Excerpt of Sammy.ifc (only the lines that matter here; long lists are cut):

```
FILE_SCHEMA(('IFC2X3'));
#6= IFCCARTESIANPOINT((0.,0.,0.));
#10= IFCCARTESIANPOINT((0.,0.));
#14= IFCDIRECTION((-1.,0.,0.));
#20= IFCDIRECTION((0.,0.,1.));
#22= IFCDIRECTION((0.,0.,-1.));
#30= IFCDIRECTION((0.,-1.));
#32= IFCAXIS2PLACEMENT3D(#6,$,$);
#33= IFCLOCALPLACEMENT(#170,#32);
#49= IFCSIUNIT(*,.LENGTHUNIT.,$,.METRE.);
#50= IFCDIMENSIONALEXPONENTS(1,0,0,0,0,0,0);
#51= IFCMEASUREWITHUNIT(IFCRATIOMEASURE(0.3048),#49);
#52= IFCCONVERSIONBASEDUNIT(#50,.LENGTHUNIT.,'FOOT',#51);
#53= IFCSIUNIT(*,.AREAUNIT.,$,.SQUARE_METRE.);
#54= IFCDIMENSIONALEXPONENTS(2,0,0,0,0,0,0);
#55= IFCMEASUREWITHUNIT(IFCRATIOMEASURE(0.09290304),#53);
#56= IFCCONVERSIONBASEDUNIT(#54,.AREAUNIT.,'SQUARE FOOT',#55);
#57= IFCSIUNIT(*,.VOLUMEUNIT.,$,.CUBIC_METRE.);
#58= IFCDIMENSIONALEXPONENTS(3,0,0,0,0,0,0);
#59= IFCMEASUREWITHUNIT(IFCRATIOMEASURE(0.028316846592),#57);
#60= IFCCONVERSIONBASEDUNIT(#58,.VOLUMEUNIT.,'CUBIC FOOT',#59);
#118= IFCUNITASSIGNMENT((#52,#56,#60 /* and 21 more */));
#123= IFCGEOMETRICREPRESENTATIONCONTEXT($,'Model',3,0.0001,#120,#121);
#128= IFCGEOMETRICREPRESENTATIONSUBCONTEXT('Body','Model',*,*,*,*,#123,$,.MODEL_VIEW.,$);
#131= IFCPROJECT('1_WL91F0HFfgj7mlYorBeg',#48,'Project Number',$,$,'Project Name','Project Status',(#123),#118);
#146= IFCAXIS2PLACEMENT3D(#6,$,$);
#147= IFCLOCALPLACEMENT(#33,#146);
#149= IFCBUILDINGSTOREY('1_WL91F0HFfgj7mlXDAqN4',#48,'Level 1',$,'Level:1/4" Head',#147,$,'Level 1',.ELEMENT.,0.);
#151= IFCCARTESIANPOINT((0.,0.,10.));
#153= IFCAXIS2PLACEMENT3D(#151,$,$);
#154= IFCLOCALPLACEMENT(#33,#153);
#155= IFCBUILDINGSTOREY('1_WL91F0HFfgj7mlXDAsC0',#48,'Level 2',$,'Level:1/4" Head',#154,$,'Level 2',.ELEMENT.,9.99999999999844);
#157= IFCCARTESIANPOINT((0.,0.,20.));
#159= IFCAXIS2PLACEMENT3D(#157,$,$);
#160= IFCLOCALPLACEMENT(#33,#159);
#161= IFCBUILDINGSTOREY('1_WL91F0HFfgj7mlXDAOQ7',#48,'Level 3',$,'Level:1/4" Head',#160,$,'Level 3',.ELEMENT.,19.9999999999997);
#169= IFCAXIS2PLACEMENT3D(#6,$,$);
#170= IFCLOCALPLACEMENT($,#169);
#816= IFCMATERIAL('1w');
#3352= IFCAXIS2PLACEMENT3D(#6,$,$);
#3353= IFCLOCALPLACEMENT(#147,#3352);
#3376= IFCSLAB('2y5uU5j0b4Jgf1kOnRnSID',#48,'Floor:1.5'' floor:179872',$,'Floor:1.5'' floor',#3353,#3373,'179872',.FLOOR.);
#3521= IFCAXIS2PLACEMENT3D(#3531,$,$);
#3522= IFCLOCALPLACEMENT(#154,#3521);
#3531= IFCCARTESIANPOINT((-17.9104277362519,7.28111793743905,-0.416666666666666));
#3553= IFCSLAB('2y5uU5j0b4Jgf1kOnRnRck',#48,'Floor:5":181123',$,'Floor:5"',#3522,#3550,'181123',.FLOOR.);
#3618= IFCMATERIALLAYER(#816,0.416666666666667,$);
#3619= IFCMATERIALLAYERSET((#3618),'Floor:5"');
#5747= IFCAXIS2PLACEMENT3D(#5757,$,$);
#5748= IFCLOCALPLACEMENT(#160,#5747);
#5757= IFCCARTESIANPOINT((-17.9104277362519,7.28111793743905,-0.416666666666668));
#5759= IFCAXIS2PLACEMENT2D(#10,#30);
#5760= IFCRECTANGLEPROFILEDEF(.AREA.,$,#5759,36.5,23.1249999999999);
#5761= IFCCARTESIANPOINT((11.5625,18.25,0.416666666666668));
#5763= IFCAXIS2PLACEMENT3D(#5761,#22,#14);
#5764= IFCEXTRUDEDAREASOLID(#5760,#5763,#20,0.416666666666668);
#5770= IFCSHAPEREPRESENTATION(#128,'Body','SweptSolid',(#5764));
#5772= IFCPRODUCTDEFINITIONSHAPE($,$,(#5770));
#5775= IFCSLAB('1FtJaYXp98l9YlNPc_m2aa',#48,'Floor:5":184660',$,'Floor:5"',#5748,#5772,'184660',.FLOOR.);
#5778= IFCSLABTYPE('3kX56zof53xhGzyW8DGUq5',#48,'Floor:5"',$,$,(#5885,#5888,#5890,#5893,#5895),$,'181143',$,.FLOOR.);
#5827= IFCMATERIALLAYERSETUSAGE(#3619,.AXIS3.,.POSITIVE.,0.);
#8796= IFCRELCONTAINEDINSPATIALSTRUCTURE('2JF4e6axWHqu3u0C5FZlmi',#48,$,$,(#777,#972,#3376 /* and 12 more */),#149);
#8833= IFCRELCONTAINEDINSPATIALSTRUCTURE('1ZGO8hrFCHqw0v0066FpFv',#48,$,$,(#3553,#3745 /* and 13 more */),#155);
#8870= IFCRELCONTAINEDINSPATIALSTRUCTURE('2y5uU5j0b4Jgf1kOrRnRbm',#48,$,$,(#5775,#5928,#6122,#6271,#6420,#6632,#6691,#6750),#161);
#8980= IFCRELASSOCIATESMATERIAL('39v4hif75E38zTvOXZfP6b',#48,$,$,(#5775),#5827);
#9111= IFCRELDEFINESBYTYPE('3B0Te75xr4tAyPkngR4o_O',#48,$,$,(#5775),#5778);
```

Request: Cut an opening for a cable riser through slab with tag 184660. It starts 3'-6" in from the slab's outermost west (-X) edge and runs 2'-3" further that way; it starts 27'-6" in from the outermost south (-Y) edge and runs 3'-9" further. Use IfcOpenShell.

```python
import numpy as np
import ifcopenshell
import ifcopenshell.api.feature
import ifcopenshell.api.geometry
import ifcopenshell.api.root
import ifcopenshell.geom
import ifcopenshell.util.placement
import ifcopenshell.util.representation
import ifcopenshell.util.shape
import ifcopenshell.util.unit

model = ifcopenshell.open("Sammy.ifc")
unit_scale = ifcopenshell.util.unit.calculate_unit_scale(model)
settings = ifcopenshell.geom.settings()


def volume(element):
    """Net volume in cubic metres, openings subtracted."""
    shape = ifcopenshell.geom.create_shape(settings, element)
    return ifcopenshell.util.shape.get_volume(shape.geometry)


slab = model.by_guid("1FtJaYXp98l9YlNPc_m2aa")
before = volume(slab)

# Extent in the slab's own axes, in metres. The edges named are its -X and -Y sides.
slab_shape = ifcopenshell.geom.create_shape(settings, slab)
vertices = ifcopenshell.util.shape.get_vertices(slab_shape.geometry)
x_min, y_min, bottom = vertices.min(axis=0)
top = vertices[:, 2].max()

opening = ifcopenshell.api.root.create_entity(model, ifc_class="IfcOpeningElement", name="Cable riser opening")
context = ifcopenshell.util.representation.get_context(model, "Model", "Body", "MODEL_VIEW")
width, depth = 0.6858, 1.143
outline = [(0.0, 0.0), (width, 0.0), (width, depth), (0.0, depth), (0.0, 0.0)]
# Overshoot both faces by 50 mm so the cut is clean.
shape = ifcopenshell.api.geometry.add_slab_representation(
    model, context=context, depth=top - bottom + 0.1, polyline=outline
)
ifcopenshell.api.geometry.assign_representation(model, product=opening, representation=shape)

matrix = ifcopenshell.util.placement.get_local_placement(slab.ObjectPlacement)
matrix[:, 3] = matrix @ np.append(np.array([x_min + 1.0668, y_min + 8.382, bottom - 0.05]) / unit_scale, 1.0)
ifcopenshell.api.geometry.edit_object_placement(model, product=opening, matrix=matrix, is_si=False)
ifcopenshell.api.feature.add_feature(model, feature=opening, element=slab)

after = volume(slab)

print(f"slab volume {before:.3f} -> {after:.3f} m3")

model.write("Sammy_rev.ifc")
```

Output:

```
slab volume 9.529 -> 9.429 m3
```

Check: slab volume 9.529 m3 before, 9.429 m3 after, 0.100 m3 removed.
